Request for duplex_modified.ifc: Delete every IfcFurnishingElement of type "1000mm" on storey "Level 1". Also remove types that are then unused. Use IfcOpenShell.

First a look at what the model holds.

```python
import ifcopenshell
import ifcopenshell.util.element

model = ifcopenshell.open("duplex_modified.ifc")
print(model.schema)
storey = next(s for s in model.by_type("IfcBuildingStorey") if s.Name == "Level 1")
furniture = [e for e in ifcopenshell.util.element.get_decomposition(storey) if e.is_a("IfcFurnishingElement")]
seen = {}
for e in furniture:
    element_type = ifcopenshell.util.element.get_type(e)
    name = element_type.Name if element_type not in (None, e) else None
    seen[name] = seen.get(name, 0) + 1
for name, count in sorted(seen.items(), key=str):
    print(count, "x", name)
```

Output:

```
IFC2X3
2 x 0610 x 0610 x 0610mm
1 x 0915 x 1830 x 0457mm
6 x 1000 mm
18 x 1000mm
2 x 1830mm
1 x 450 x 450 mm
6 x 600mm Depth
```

```python
import ifcopenshell
import ifcopenshell.api.root
import ifcopenshell.util.element

model = ifcopenshell.open("duplex_modified.ifc")

storey = next(s for s in model.by_type("IfcBuildingStorey") if s.Name == "Level 1")
furniture = [e for e in ifcopenshell.util.element.get_decomposition(storey) if e.is_a("IfcFurnishingElement")]
targets = [e for e in furniture if (t := ifcopenshell.util.element.get_type(e)) not in (None, e) and t.Name == "1000mm"]
types = {ifcopenshell.util.element.get_type(e) for e in targets} - {None, *targets}

for e in targets:
    ifcopenshell.api.root.remove_product(model, product=e)
print(len(targets), "removed")

unused = [t for t in types if not ifcopenshell.util.element.get_types(t)]
for t in unused:
    ifcopenshell.api.root.remove_product(model, product=t)
print(len(unused), "unused types removed")

model.write("duplex_modified_v2.ifc")
```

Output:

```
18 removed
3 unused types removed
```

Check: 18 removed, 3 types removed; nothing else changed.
